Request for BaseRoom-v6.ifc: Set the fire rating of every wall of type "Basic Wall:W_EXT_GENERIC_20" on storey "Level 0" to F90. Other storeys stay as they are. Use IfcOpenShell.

First a look at what the model holds.

```python
import ifcopenshell
import ifcopenshell.util.element

model = ifcopenshell.open("BaseRoom-v6.ifc")
print(model.schema)
storey = next(s for s in model.by_type("IfcBuildingStorey") if s.Name == "Level 0")
walls = [e for e in ifcopenshell.util.element.get_decomposition(storey) if e.is_a("IfcWall")]
seen = {}
for e in walls:
    element_type = ifcopenshell.util.element.get_type(e)
    key = (element_type.Name if element_type != e and element_type else None, ifcopenshell.util.element.get_pset(e, "Pset_WallCommon", "FireRating"))
    seen[key] = seen.get(key, 0) + 1
for (name, value), count in sorted(seen.items(), key=str):
    print(count, "x", name, "|", value)
```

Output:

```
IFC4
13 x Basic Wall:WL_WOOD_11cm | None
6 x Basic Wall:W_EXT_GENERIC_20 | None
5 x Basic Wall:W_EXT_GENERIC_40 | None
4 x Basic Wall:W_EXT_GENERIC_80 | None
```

```python
import ifcopenshell
import ifcopenshell.api.pset
import ifcopenshell.util.element

model = ifcopenshell.open("BaseRoom-v6.ifc")

storey = next(s for s in model.by_type("IfcBuildingStorey") if s.Name == "Level 0")
walls = [e for e in ifcopenshell.util.element.get_decomposition(storey) if e.is_a("IfcWall")]

count = 0
for e in walls:
    element_type = ifcopenshell.util.element.get_type(e)
    if element_type in (None, e) or element_type.Name != "Basic Wall:W_EXT_GENERIC_20":
        continue
    # add_pset returns the element's existing set when there is one.
    pset = ifcopenshell.api.pset.add_pset(model, product=e, name="Pset_WallCommon")
    ifcopenshell.api.pset.edit_pset(model, pset=pset, properties={"FireRating": "F90"})
    count += 1

print(count, "walls updated")

model.write("BaseRoom-v6_edited.ifc")
```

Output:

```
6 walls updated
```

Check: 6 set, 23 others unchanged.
